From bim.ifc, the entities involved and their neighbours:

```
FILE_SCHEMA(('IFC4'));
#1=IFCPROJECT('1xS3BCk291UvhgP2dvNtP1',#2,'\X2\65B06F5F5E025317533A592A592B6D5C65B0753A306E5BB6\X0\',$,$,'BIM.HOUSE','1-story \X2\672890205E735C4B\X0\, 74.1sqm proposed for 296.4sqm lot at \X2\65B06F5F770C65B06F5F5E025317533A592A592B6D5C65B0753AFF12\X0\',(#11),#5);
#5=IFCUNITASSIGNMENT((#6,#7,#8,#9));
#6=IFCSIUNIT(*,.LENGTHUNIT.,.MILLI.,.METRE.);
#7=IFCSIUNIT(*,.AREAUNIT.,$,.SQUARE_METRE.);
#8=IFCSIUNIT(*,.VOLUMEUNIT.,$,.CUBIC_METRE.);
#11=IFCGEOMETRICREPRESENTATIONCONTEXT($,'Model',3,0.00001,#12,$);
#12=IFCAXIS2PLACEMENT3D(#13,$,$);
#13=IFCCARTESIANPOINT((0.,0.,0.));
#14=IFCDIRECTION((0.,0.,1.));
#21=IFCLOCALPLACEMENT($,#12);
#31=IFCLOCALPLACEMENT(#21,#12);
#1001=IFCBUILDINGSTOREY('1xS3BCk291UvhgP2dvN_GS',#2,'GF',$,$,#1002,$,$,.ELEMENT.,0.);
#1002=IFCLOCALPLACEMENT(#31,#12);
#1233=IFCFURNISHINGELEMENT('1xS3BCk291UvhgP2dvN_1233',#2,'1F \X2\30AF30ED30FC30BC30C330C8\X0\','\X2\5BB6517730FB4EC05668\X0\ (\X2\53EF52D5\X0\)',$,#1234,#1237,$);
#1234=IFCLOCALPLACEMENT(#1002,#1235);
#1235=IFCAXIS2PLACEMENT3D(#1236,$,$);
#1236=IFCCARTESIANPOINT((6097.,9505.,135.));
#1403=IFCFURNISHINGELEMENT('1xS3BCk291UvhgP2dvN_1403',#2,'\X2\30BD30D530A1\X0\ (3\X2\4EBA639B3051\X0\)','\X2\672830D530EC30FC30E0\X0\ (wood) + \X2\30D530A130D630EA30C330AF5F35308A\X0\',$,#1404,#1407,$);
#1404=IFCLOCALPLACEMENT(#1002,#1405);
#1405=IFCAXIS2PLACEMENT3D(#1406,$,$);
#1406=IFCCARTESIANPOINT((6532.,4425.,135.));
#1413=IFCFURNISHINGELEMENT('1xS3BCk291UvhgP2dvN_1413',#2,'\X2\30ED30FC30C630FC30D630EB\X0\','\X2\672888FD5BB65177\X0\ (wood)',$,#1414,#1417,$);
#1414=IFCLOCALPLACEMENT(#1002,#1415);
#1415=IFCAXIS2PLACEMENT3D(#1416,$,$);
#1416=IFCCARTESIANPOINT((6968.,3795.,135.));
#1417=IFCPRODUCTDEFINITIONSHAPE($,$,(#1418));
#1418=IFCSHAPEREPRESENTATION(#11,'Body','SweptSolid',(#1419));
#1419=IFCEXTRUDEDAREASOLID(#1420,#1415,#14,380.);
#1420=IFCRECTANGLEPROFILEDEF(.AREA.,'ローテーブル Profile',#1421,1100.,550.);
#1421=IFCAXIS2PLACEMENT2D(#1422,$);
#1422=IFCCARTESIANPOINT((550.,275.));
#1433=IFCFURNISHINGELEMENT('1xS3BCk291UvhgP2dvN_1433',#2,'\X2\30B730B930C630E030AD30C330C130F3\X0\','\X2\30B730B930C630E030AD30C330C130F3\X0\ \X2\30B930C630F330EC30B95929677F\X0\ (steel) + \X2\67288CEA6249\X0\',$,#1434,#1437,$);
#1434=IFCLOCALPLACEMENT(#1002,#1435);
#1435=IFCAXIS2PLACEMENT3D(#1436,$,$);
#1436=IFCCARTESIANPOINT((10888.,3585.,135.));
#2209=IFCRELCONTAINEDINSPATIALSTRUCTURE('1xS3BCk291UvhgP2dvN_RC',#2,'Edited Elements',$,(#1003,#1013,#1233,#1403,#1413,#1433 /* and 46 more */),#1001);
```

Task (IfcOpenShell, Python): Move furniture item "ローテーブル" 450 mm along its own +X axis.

```python
import ifcopenshell
import ifcopenshell.api.geometry
import ifcopenshell.util.placement

model = ifcopenshell.open("bim.ifc")

item = model.by_guid("1xS3BCk291UvhgP2dvN_1413")
matrix = ifcopenshell.util.placement.get_local_placement(item.ObjectPlacement)
matrix[:3, 3] += matrix[:3, 0] * 450.0
ifcopenshell.api.geometry.edit_object_placement(model, product=item, matrix=matrix, is_si=False)

print(ifcopenshell.util.placement.get_local_placement(item.ObjectPlacement).round(3) + 0.0)

model.write("bim-out.ifc")
```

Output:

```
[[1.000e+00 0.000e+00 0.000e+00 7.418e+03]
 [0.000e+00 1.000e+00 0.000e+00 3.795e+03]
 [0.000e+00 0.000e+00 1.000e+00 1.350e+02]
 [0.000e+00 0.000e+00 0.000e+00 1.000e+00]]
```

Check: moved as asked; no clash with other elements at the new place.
